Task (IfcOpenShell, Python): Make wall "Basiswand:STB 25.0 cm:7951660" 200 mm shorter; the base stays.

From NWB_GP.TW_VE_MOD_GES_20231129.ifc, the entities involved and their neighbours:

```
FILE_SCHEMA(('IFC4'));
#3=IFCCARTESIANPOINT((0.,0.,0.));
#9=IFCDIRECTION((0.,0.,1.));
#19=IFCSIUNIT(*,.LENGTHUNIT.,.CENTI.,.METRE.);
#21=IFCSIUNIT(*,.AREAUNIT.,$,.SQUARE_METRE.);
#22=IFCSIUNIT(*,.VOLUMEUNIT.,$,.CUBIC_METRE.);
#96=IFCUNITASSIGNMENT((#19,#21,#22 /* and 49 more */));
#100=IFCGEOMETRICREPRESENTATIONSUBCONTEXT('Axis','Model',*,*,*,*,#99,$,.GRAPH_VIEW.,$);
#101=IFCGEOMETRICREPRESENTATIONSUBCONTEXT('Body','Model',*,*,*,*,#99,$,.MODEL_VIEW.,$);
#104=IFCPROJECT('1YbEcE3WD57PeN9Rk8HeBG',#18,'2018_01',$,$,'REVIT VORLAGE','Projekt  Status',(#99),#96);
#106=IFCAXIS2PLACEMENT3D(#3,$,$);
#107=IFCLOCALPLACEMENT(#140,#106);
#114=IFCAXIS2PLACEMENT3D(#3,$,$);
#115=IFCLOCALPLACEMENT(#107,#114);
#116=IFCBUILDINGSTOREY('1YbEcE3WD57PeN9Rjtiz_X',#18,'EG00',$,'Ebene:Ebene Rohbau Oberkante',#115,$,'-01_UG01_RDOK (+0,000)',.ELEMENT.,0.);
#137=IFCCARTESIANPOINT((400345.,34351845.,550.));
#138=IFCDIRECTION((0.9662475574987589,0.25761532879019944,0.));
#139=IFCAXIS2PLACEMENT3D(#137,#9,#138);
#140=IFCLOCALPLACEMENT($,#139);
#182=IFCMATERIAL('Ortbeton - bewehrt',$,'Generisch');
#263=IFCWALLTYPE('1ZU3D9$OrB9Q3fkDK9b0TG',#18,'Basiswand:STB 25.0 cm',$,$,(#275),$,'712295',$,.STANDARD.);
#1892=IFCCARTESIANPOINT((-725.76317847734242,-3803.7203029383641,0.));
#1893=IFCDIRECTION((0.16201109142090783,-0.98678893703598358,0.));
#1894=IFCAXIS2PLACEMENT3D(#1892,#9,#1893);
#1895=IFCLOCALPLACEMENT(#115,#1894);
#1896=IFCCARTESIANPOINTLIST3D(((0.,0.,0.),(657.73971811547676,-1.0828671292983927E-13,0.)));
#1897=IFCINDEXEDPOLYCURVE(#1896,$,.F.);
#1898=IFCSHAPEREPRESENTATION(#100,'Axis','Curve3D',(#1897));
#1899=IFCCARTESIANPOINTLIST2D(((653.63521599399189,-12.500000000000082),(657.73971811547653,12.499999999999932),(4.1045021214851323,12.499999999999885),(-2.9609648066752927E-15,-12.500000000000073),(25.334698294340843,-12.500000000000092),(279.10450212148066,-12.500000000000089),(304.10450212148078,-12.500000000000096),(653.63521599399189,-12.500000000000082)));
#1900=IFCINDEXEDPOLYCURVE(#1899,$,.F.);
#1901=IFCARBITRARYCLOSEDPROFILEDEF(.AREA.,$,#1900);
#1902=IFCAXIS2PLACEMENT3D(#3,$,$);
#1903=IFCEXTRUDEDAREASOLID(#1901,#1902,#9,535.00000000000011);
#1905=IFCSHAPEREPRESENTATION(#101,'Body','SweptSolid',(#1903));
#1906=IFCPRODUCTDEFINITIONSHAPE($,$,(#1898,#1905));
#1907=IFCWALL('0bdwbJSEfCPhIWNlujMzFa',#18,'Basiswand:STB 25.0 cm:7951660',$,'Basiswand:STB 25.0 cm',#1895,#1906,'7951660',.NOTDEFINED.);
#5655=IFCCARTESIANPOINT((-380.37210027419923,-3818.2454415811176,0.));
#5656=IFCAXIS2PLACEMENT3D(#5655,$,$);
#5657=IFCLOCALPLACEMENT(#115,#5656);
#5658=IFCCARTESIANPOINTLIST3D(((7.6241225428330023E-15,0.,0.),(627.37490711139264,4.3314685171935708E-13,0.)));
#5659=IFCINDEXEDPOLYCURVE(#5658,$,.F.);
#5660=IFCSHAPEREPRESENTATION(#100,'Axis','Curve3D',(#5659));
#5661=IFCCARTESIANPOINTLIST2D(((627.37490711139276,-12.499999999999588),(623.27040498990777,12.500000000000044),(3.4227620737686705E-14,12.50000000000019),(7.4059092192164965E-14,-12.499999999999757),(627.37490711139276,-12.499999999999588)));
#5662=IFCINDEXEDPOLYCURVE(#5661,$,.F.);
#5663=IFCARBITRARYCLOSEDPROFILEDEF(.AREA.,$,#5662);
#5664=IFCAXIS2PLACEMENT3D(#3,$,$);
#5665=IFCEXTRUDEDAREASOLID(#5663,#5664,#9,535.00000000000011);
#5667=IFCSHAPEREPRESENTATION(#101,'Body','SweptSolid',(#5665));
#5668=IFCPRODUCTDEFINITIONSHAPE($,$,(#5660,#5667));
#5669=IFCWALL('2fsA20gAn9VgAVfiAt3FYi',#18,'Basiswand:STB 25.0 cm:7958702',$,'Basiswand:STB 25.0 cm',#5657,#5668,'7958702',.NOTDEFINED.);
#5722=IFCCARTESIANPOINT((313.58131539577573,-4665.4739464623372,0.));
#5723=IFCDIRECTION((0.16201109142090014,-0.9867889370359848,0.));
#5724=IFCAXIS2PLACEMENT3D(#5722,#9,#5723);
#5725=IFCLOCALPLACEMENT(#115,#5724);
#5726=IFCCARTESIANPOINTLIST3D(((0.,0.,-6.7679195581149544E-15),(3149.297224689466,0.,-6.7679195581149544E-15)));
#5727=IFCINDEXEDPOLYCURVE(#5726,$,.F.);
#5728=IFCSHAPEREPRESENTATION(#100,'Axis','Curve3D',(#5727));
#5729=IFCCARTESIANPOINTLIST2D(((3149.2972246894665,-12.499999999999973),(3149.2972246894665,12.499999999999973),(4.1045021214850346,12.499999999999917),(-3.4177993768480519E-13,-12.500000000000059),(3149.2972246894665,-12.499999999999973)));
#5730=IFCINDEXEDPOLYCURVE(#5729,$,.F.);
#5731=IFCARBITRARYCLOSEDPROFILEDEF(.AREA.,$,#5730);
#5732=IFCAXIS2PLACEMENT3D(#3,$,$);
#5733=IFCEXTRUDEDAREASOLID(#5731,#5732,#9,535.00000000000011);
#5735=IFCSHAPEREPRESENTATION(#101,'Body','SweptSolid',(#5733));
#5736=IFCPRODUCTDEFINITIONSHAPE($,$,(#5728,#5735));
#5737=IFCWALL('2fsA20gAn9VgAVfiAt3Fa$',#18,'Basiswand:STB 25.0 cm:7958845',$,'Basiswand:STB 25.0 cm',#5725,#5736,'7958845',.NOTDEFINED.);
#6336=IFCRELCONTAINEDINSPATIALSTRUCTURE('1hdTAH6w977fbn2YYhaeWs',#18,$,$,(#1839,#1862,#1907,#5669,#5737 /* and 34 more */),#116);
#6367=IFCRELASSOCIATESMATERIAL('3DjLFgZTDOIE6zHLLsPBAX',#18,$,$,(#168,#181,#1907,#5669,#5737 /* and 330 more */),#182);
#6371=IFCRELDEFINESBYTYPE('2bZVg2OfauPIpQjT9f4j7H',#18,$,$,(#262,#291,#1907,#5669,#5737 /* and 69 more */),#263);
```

```python
import ifcopenshell
import ifcopenshell.geom
import ifcopenshell.util.representation
import ifcopenshell.util.shape
import ifcopenshell.util.unit

model = ifcopenshell.open("NWB_GP.TW_VE_MOD_GES_20231129.ifc")
unit_scale = ifcopenshell.util.unit.calculate_unit_scale(model)
settings = ifcopenshell.geom.settings()


def volume(element):
    """Net volume in cubic metres, openings subtracted."""
    shape = ifcopenshell.geom.create_shape(settings, element)
    return ifcopenshell.util.shape.get_volume(shape.geometry)


wall = model.by_guid("0bdwbJSEfCPhIWNlujMzFa")
before = volume(wall)

body = ifcopenshell.util.representation.get_representation(wall, "Model", "Body")
solid = body.Items[0]
old_height = solid.Depth
solid.Depth -= 0.2 / unit_scale
after = volume(wall)

print(f"height {old_height:g} -> {solid.Depth:g}, volume {before:.3f} -> {after:.3f} m3")

model.write("NWB_GP.TW_VE_MOD_GES_20231129-out.ifc")
```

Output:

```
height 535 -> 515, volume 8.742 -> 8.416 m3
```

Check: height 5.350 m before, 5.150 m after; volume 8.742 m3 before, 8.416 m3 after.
